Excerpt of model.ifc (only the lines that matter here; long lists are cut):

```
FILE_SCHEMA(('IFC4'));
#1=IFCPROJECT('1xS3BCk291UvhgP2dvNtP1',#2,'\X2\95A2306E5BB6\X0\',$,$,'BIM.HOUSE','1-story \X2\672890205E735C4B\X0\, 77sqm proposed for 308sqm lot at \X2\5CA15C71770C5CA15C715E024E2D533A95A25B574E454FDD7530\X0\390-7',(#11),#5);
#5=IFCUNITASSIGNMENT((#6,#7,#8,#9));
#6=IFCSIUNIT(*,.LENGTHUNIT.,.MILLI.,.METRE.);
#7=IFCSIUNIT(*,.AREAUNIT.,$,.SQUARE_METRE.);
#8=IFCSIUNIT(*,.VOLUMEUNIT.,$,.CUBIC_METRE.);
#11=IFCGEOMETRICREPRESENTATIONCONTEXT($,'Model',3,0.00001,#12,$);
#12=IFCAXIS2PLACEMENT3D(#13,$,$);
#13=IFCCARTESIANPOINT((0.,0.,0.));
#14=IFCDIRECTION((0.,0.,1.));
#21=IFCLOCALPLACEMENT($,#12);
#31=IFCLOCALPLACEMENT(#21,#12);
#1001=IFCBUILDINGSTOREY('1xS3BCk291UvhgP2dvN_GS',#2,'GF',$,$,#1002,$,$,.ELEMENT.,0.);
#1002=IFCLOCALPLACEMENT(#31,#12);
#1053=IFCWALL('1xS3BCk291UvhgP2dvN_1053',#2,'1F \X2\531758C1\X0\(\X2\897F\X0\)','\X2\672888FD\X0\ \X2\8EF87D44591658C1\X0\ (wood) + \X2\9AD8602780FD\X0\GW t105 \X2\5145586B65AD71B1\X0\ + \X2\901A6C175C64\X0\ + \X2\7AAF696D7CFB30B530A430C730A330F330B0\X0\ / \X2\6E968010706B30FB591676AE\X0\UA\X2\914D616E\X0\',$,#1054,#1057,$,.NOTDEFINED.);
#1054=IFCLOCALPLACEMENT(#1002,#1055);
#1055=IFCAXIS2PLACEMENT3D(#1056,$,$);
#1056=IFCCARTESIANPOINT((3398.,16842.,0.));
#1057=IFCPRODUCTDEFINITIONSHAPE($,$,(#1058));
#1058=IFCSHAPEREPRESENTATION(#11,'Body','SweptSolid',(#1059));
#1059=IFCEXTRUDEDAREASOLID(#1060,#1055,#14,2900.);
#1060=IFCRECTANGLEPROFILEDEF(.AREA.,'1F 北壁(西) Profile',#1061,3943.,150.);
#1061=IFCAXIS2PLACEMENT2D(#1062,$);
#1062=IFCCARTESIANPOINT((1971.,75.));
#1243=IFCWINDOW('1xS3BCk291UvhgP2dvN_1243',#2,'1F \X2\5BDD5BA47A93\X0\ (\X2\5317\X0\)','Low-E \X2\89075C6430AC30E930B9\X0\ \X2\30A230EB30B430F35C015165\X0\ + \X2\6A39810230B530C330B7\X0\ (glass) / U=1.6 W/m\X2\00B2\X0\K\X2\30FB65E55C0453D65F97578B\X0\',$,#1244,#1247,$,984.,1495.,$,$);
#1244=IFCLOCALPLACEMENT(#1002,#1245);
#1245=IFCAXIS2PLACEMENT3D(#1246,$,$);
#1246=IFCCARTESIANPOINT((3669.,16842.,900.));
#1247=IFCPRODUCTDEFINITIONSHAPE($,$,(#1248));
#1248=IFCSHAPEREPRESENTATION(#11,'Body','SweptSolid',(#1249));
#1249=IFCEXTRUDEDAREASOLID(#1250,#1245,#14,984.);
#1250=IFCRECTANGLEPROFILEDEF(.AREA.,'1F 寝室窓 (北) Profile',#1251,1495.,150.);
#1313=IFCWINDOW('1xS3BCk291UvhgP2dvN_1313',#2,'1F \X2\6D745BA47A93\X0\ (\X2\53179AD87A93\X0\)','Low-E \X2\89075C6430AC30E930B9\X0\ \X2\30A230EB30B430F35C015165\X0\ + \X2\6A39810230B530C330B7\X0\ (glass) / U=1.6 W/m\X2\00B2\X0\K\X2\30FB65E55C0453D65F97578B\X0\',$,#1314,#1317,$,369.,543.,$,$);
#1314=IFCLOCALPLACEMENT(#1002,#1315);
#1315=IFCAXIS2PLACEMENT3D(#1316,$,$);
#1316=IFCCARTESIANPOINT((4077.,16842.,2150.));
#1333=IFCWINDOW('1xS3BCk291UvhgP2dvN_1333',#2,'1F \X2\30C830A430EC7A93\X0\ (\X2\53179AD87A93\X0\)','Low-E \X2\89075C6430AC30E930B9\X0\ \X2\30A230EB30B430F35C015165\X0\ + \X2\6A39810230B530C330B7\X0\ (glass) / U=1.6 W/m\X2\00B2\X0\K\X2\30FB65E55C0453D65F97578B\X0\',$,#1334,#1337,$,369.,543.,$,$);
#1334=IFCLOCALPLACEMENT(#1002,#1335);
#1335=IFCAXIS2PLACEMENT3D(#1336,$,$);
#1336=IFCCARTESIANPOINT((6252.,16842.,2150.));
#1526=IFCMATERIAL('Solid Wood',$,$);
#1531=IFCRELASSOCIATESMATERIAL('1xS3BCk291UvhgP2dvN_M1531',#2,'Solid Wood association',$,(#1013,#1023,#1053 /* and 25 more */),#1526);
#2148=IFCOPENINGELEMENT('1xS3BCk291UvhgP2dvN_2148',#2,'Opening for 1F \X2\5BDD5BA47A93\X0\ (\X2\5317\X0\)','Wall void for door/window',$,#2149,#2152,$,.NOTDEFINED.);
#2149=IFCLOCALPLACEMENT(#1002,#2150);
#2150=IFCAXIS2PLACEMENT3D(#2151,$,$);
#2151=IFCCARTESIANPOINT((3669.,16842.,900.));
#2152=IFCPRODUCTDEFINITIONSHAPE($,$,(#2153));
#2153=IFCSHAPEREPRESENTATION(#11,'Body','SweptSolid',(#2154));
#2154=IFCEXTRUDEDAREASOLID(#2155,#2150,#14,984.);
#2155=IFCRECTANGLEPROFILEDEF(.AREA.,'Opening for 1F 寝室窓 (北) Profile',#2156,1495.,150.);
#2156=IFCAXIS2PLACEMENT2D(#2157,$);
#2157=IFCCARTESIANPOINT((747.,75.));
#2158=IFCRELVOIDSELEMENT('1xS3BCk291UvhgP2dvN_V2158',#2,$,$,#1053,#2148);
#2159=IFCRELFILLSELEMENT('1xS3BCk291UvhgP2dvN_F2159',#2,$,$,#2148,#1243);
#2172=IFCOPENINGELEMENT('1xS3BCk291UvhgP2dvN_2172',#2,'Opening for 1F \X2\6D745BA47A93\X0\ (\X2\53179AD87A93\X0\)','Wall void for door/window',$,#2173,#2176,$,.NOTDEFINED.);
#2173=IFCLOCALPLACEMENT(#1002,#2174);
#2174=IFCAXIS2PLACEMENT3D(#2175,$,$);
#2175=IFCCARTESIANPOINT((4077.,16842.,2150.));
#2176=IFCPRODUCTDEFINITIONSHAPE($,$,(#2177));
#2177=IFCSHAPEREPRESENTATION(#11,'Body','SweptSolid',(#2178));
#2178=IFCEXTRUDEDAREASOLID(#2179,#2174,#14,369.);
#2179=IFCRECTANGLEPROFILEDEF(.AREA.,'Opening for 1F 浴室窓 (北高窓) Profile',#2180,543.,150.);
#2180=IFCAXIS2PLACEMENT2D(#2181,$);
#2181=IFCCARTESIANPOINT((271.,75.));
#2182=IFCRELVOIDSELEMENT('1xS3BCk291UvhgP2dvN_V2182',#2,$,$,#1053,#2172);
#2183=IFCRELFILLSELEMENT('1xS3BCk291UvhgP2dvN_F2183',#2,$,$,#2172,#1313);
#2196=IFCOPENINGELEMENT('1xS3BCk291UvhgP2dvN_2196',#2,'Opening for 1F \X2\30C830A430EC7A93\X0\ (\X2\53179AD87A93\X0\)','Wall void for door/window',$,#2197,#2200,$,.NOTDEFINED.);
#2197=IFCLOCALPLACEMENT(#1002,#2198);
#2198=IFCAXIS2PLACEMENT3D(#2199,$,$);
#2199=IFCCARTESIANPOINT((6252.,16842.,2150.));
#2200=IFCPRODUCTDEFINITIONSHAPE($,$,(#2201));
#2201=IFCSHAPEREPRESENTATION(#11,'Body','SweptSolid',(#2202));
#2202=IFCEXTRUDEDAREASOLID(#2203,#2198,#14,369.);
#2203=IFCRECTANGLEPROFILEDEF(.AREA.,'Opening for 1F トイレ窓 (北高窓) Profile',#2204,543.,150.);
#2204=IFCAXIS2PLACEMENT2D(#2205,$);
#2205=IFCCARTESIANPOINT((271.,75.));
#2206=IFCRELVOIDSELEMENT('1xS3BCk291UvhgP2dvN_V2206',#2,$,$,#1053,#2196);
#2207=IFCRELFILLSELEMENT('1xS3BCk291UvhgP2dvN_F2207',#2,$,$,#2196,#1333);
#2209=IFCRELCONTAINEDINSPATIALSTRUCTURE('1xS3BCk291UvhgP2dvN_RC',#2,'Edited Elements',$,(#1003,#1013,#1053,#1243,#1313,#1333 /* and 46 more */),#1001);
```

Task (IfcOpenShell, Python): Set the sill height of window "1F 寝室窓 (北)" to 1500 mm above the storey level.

```python
import numpy as np
import ifcopenshell
import ifcopenshell.api.geometry
import ifcopenshell.geom
import ifcopenshell.util.element
import ifcopenshell.util.placement
import ifcopenshell.util.shape
import ifcopenshell.util.unit

model = ifcopenshell.open("model.ifc")
unit_scale = ifcopenshell.util.unit.calculate_unit_scale(model)

window = model.by_id(1243)
opening = window.FillsVoids[0].RelatingOpeningElement
storey = ifcopenshell.util.element.get_container(window, ifc_class="IfcBuildingStorey")
level = ifcopenshell.util.placement.get_local_placement(storey.ObjectPlacement)[2, 3]

# The opening's origin need not be at the sill, so measure its lowest point.
shape = ifcopenshell.geom.create_shape(ifcopenshell.geom.settings(), opening)
bottom = ifcopenshell.util.shape.get_shape_bottom_elevation(shape, shape.geometry) / unit_scale
dz = level + 1500.0 - bottom

shift = np.array([0.0, 0.0, dz])
# The window is not placed relative to its opening, so move both.
for product in (opening, window):
    matrix = ifcopenshell.util.placement.get_local_placement(product.ObjectPlacement)
    matrix[:3, 3] += shift
    ifcopenshell.api.geometry.edit_object_placement(model, product=product, matrix=matrix, is_si=False)

print(f"moved by {dz * unit_scale:+.3f} m")

model.write("model_edited.ifc")
```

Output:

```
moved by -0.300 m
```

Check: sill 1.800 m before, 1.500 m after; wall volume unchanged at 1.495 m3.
